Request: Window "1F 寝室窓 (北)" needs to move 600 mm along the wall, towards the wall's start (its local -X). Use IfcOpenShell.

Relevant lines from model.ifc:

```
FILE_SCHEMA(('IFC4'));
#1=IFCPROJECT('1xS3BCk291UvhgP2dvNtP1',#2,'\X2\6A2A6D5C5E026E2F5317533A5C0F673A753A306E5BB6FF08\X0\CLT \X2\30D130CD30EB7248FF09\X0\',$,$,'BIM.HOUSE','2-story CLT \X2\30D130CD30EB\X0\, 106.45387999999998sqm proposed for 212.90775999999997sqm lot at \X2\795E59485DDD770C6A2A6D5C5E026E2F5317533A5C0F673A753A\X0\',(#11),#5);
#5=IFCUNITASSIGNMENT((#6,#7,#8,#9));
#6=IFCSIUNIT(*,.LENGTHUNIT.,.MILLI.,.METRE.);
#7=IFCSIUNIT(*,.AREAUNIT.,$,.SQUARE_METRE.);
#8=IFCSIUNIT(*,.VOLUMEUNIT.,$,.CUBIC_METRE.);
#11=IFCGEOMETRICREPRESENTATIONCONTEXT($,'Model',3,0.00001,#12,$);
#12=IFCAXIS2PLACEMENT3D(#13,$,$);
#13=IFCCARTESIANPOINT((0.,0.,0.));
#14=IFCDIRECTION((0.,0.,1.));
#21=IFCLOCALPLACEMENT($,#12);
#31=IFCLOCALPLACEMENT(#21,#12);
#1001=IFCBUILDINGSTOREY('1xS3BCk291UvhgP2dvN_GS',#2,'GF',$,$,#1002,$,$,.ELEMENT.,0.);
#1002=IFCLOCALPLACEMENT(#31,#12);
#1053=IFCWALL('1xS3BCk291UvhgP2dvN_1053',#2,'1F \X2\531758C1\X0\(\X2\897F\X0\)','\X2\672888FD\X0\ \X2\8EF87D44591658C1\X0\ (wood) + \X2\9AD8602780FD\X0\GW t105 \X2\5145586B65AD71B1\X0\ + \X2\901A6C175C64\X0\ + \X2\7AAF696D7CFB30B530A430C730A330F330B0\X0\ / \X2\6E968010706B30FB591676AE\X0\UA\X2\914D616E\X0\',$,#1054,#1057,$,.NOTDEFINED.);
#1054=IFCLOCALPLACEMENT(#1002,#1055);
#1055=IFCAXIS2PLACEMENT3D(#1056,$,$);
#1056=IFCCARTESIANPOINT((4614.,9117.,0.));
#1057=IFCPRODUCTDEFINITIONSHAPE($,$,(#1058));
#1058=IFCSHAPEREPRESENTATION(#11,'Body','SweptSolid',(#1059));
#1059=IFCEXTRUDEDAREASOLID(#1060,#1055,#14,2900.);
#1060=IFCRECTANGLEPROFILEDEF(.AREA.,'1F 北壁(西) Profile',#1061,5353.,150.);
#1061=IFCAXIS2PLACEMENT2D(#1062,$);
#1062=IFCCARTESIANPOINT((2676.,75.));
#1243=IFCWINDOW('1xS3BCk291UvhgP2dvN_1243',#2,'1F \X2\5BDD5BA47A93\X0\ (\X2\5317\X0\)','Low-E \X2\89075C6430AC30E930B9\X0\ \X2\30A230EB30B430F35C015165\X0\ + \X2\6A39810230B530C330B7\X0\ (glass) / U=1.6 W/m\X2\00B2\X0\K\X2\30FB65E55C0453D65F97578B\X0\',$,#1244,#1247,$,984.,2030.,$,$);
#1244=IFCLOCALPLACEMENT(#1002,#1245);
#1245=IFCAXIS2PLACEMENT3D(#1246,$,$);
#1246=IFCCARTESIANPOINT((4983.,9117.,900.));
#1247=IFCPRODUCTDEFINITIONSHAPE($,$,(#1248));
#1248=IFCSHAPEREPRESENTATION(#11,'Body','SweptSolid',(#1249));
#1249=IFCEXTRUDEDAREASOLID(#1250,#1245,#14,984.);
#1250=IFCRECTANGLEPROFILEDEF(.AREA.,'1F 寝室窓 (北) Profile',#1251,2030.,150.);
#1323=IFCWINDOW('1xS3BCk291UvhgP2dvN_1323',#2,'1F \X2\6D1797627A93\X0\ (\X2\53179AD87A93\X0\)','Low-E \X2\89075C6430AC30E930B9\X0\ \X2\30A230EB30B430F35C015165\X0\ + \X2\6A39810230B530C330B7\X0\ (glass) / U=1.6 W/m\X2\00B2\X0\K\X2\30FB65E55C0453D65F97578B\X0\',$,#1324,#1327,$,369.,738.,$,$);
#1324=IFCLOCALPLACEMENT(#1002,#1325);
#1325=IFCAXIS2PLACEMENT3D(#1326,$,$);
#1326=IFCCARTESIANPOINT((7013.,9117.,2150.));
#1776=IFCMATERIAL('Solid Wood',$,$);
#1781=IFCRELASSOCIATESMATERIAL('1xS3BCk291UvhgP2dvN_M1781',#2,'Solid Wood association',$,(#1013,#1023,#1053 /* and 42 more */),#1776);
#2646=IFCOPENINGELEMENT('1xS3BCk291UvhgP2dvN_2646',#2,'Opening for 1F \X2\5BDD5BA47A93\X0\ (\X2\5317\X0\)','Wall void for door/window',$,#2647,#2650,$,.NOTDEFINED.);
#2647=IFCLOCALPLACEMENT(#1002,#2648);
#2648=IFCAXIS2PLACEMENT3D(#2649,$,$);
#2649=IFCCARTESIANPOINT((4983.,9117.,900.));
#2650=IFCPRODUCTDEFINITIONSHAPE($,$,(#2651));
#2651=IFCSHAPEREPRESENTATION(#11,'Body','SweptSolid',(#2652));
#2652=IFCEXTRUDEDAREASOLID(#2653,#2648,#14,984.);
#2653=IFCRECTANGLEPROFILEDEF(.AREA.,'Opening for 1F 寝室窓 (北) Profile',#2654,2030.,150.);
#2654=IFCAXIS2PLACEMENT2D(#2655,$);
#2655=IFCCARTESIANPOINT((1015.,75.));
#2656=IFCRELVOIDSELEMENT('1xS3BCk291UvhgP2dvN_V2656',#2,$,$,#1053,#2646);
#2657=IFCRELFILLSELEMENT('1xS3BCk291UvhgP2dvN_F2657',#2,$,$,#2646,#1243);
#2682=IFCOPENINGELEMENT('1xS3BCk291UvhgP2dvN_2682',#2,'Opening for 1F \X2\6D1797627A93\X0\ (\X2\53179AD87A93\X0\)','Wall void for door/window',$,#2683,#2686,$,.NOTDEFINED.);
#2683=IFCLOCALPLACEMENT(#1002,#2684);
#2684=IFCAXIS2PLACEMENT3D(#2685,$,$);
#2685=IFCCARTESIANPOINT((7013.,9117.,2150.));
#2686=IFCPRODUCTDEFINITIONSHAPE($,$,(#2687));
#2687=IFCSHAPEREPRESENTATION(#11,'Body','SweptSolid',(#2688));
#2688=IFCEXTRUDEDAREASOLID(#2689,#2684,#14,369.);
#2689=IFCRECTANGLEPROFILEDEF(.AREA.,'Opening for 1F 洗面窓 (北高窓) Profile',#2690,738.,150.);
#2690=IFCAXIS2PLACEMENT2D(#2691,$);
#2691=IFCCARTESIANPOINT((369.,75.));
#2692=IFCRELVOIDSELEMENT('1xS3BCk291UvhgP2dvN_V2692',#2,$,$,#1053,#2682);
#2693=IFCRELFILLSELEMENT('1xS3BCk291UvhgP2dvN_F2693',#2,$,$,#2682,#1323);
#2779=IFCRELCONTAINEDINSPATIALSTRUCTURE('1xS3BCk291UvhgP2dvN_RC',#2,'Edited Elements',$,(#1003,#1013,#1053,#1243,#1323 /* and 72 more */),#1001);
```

```python
import ifcopenshell
import ifcopenshell.api.geometry
import ifcopenshell.util.placement

model = ifcopenshell.open("model.ifc")

window = model.by_guid("1xS3BCk291UvhgP2dvN_1243")
opening = window.FillsVoids[0].RelatingOpeningElement
wall = opening.VoidsElements[0].RelatingBuildingElement

wall_matrix = ifcopenshell.util.placement.get_local_placement(wall.ObjectPlacement)
shift = wall_matrix[:3, 0] * -600.0
before = ifcopenshell.util.placement.get_local_placement(window.ObjectPlacement)[:3, 3].copy()

# The window is not placed relative to its opening, so move both.
for product in (opening, window):
    matrix = ifcopenshell.util.placement.get_local_placement(product.ObjectPlacement)
    matrix[:3, 3] += shift
    ifcopenshell.api.geometry.edit_object_placement(model, product=product, matrix=matrix, is_si=False)

after = ifcopenshell.util.placement.get_local_placement(window.ObjectPlacement)[:3, 3]
print("window moved by", (after - before).round(3) + 0.0)

model.write("model_updated.ifc")
```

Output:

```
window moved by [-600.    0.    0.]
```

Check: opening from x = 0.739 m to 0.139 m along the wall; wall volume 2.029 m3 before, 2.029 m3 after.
